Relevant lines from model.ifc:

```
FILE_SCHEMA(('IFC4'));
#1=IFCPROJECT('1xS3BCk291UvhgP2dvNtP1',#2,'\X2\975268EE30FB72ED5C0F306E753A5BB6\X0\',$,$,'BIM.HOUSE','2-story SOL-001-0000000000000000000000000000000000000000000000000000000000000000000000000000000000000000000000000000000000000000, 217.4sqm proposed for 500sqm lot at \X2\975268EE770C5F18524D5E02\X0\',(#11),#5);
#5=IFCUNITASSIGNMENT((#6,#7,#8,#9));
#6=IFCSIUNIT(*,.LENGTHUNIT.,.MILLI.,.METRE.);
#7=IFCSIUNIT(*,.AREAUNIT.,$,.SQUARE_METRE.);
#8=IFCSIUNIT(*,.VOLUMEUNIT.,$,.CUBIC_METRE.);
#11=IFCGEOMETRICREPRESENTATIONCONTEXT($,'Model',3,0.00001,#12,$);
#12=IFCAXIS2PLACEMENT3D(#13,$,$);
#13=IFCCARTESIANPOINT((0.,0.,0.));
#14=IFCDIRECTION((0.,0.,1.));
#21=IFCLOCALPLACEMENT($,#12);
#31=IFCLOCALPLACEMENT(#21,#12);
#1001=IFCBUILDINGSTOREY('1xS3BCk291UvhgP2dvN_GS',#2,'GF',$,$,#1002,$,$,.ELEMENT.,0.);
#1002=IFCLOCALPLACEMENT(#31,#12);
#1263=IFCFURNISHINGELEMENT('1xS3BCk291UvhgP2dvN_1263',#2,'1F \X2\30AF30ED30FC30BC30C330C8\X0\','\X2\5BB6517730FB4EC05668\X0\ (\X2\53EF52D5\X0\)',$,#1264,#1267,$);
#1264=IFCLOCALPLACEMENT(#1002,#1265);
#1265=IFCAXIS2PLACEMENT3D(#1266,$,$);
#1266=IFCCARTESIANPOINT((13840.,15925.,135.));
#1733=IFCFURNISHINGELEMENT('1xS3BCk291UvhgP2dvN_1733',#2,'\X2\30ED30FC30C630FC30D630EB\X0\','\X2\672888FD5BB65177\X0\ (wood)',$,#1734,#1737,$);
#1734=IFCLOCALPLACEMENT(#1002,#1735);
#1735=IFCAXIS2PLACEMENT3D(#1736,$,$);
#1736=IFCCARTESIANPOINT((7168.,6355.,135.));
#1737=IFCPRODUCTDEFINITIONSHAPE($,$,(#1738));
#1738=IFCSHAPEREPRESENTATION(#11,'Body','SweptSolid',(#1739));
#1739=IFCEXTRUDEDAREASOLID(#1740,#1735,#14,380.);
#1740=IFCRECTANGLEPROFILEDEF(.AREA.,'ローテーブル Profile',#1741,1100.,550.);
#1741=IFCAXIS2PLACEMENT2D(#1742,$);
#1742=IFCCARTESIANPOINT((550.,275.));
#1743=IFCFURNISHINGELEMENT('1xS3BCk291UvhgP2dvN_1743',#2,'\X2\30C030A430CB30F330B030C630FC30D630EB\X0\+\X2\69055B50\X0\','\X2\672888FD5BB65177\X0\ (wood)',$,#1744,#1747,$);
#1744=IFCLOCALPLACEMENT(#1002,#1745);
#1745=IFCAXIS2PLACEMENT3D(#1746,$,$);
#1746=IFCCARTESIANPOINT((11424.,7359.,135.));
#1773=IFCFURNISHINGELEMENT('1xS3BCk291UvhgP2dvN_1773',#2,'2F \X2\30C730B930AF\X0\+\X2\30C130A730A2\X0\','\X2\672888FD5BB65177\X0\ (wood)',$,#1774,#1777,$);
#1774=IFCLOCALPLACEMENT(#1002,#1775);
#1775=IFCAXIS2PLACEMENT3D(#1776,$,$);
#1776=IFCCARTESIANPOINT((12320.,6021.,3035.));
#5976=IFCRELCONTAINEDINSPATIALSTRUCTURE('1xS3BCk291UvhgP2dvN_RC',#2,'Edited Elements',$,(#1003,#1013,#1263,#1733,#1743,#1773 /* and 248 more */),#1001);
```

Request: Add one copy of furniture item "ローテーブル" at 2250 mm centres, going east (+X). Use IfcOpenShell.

```python
import numpy as np
import ifcopenshell
import ifcopenshell.api.geometry
import ifcopenshell.api.root
import ifcopenshell.util.element
import ifcopenshell.util.placement
import ifcopenshell.util.unit

model = ifcopenshell.open("model.ifc")
unit_scale = ifcopenshell.util.unit.calculate_unit_scale(model)


def reuse_history(source, copy):
    """copy_class also copies each property set's owner history, people and application; keep the originals."""
    for rel in copy.IsDefinedBy:
        if rel.is_a("IfcRelDefinesByProperties") and (history := rel.RelatingPropertyDefinition.OwnerHistory):
            rel.RelatingPropertyDefinition.OwnerHistory = source.OwnerHistory
            ifcopenshell.util.element.remove_deep2(model, history)


source = model.by_guid("1xS3BCk291UvhgP2dvN_1733")
base = ifcopenshell.util.placement.get_local_placement(source.ObjectPlacement)
step = np.array([1.0, 0.0, 0.0]) * 2.25 / unit_scale

for i in range(1, 2):
    copy = ifcopenshell.api.root.copy_class(model, product=source)
    copy.Representation = ifcopenshell.util.element.copy_deep(
        model, source.Representation, exclude=["IfcGeometricRepresentationContext", "IfcRepresentationMap"]
    )
    reuse_history(source, copy)
    matrix = base.copy()
    matrix[:3, 3] += i * step
    print("added at", matrix[:3, 3].round(3) + 0.0)
    ifcopenshell.api.geometry.edit_object_placement(model, product=copy, matrix=matrix, is_si=False)

model.write("model_rev.ifc")
```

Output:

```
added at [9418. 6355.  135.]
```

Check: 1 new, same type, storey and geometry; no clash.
